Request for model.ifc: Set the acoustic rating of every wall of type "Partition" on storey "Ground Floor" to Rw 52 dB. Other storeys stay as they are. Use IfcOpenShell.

First a look at what the model holds.

```python
import ifcopenshell
import ifcopenshell.util.element

model = ifcopenshell.open("model.ifc")
print(model.schema)
storey = next(s for s in model.by_type("IfcBuildingStorey") if s.Name == "Ground Floor")
walls = [e for e in ifcopenshell.util.element.get_decomposition(storey) if e.is_a("IfcWall")]
seen = {}
for e in walls:
    element_type = ifcopenshell.util.element.get_type(e)
    key = (element_type.Name if element_type != e and element_type else None, ifcopenshell.util.element.get_pset(e, "Pset_WallCommon", "AcousticRating"))
    seen[key] = seen.get(key, 0) + 1
for (name, value), count in sorted(seen.items(), key=str):
    print(count, "x", name, "|", value)
```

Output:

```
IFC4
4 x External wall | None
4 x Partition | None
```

```python
import ifcopenshell
import ifcopenshell.api.pset
import ifcopenshell.util.element

model = ifcopenshell.open("model.ifc")

storey = next(s for s in model.by_type("IfcBuildingStorey") if s.Name == "Ground Floor")
walls = [e for e in ifcopenshell.util.element.get_decomposition(storey) if e.is_a("IfcWall")]

count = 0
for e in walls:
    element_type = ifcopenshell.util.element.get_type(e)
    if element_type in (None, e) or element_type.Name != "Partition":
        continue
    # add_pset returns the element's existing set when there is one.
    pset = ifcopenshell.api.pset.add_pset(model, product=e, name="Pset_WallCommon")
    ifcopenshell.api.pset.edit_pset(model, pset=pset, properties={"AcousticRating": "Rw 52 dB"})
    count += 1

print(count, "walls updated")

model.write("model-out.ifc")
```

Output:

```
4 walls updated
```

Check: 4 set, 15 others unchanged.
